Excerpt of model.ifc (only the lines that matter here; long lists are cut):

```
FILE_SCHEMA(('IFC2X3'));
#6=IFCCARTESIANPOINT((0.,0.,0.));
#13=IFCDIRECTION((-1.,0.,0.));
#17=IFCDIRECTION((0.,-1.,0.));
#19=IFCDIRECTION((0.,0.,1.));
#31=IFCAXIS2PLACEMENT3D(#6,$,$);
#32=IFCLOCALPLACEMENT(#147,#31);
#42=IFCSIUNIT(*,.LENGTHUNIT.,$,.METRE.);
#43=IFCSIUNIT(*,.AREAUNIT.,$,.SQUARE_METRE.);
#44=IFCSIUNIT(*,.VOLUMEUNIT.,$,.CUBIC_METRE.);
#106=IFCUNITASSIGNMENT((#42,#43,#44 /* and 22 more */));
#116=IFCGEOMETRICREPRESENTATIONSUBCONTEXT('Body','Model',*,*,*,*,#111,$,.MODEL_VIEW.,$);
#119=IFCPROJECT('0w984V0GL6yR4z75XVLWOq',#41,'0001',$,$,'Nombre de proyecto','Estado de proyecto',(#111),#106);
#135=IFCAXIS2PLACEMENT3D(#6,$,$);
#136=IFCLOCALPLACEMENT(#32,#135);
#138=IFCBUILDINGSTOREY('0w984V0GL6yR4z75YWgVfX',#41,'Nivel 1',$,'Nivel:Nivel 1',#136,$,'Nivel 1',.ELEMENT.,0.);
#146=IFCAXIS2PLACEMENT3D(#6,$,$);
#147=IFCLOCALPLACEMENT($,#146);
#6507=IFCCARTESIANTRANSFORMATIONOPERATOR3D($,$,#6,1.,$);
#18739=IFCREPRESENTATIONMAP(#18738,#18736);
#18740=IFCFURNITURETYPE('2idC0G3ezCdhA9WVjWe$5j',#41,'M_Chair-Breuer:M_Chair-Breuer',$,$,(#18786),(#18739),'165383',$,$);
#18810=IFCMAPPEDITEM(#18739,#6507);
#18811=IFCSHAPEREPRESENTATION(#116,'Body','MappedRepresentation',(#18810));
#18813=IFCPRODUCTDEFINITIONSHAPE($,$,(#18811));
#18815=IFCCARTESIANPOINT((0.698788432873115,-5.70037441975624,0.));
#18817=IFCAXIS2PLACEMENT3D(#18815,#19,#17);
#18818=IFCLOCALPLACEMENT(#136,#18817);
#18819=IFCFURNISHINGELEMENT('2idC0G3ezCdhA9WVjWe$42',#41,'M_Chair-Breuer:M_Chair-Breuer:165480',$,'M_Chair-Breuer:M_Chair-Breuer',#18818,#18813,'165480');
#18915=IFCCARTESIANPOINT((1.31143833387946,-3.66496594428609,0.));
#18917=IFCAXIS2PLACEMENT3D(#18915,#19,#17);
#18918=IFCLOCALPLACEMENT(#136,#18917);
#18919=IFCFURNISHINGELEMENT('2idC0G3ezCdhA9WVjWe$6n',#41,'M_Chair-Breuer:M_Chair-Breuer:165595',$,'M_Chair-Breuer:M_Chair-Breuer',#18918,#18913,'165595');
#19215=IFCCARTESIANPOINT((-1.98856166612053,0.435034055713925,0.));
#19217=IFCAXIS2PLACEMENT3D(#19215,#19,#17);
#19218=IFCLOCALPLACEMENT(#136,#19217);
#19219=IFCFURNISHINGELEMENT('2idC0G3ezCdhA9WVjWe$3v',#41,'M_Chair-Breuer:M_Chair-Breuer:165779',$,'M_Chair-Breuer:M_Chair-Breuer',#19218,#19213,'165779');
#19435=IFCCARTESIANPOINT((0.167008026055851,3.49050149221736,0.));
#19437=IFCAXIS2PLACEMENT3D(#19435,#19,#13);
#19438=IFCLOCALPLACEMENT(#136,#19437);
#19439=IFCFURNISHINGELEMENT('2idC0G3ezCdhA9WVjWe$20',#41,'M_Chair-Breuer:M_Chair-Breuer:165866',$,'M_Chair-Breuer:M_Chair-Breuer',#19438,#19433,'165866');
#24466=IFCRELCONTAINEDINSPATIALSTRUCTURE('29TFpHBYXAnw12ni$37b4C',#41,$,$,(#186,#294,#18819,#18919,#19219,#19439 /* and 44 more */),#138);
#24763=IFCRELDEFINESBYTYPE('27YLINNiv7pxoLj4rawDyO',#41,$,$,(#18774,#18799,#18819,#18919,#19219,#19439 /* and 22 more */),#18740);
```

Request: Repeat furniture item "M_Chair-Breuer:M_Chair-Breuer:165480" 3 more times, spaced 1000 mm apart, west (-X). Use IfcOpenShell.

```python
import numpy as np
import ifcopenshell
import ifcopenshell.api.geometry
import ifcopenshell.api.root
import ifcopenshell.util.element
import ifcopenshell.util.placement
import ifcopenshell.util.unit

model = ifcopenshell.open("model.ifc")
unit_scale = ifcopenshell.util.unit.calculate_unit_scale(model)


def reuse_history(source, copy):
    """copy_class also copies each property set's owner history, people and application; keep the originals."""
    for rel in copy.IsDefinedBy:
        if rel.is_a("IfcRelDefinesByProperties") and (history := rel.RelatingPropertyDefinition.OwnerHistory):
            rel.RelatingPropertyDefinition.OwnerHistory = source.OwnerHistory
            ifcopenshell.util.element.remove_deep2(model, history)


source = model.by_guid("2idC0G3ezCdhA9WVjWe$42")
base = ifcopenshell.util.placement.get_local_placement(source.ObjectPlacement)
step = np.array([-1.0, 0.0, 0.0]) * 1 / unit_scale

for i in range(1, 4):
    copy = ifcopenshell.api.root.copy_class(model, product=source)
    copy.Representation = ifcopenshell.util.element.copy_deep(
        model, source.Representation, exclude=["IfcGeometricRepresentationContext", "IfcRepresentationMap"]
    )
    copy.Name = "M_Chair-Breuer:M_Chair-Breuer"
    copy.Tag = None
    reuse_history(source, copy)
    matrix = base.copy()
    matrix[:3, 3] += i * step
    print("added at", matrix[:3, 3].round(3) + 0.0)
    ifcopenshell.api.geometry.edit_object_placement(model, product=copy, matrix=matrix, is_si=False)

model.write("model_rev.ifc")
```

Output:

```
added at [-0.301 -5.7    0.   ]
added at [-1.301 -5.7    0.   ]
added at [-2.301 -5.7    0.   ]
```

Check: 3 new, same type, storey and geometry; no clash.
